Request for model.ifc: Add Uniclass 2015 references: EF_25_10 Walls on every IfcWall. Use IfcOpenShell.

First a look at what the model holds.

```python
import ifcopenshell

model = ifcopenshell.open("model.ifc")
print(model.schema)
print("classifications:", [c.Name for c in model.by_type("IfcClassification")])
for ifc_class in ("IfcDoor", "IfcRoof", "IfcStair", "IfcWall", "IfcWindow"):
    print(ifc_class, len(model.by_type(ifc_class)))
```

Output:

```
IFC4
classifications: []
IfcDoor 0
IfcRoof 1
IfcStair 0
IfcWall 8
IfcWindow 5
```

```python
import ifcopenshell
import ifcopenshell.api.classification

model = ifcopenshell.open("model.ifc")

system = ifcopenshell.api.classification.add_classification(model, classification="Uniclass 2015")

codes = {
    "IfcWall": ("EF_25_10", "Walls"),
}
for ifc_class, (code, name) in codes.items():
    products = model.by_type(ifc_class)
    ifcopenshell.api.classification.add_reference(
        model, products=products, classification=system, identification=code, name=name
    )
    print(code, len(products))

model.write("model-out.ifc")
```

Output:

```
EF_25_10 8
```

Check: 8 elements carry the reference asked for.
